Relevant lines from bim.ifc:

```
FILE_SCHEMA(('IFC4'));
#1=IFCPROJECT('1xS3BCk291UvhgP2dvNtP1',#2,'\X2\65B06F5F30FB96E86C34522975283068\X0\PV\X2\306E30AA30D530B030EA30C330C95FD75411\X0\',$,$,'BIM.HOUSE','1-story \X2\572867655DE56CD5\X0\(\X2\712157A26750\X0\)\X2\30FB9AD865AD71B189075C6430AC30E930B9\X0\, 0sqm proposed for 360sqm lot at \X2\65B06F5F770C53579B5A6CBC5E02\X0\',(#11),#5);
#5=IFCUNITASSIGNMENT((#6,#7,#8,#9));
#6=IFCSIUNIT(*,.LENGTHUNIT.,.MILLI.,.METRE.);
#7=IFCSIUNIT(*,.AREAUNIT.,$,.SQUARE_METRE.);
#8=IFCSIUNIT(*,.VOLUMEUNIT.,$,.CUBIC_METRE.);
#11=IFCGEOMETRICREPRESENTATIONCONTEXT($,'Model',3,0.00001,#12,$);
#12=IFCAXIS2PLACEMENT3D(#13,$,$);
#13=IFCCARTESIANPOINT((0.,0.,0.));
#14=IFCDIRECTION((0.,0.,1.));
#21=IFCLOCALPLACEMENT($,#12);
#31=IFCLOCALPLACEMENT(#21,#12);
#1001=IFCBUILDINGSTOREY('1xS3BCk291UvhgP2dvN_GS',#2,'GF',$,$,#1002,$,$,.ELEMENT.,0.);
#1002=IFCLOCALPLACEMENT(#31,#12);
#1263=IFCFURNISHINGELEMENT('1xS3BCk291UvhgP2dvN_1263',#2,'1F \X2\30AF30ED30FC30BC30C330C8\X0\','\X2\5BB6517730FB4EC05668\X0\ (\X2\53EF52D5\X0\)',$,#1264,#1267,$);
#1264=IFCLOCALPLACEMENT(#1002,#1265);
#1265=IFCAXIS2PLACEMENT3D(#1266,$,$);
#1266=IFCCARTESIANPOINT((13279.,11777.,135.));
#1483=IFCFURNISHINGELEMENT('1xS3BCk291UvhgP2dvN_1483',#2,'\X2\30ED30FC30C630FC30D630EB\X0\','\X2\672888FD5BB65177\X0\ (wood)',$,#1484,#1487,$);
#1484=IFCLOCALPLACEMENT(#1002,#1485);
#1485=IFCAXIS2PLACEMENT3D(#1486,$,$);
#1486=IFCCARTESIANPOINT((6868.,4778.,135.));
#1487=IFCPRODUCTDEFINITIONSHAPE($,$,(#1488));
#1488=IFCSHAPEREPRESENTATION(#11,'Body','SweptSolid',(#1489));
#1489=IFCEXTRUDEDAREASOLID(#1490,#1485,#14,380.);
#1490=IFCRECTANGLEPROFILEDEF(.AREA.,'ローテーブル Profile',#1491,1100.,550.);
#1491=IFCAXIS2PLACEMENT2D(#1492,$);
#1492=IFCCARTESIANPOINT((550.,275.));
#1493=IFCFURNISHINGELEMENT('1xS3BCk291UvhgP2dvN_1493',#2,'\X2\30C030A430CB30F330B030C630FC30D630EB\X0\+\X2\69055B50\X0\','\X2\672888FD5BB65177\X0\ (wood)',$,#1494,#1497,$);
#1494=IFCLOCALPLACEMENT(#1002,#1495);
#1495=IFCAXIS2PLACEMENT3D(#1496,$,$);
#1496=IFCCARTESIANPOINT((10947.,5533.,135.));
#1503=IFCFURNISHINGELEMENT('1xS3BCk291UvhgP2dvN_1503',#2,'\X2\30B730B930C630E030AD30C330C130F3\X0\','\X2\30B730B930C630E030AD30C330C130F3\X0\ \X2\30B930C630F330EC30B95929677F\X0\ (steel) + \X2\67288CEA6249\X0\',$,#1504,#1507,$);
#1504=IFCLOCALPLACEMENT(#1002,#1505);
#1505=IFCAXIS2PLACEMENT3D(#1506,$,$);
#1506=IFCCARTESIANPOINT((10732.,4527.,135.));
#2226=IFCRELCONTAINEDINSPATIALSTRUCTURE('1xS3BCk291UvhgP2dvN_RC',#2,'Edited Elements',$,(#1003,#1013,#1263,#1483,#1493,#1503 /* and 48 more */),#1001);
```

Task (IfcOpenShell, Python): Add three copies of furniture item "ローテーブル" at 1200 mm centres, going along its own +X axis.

```python
import ifcopenshell
import ifcopenshell.api.geometry
import ifcopenshell.api.root
import ifcopenshell.util.element
import ifcopenshell.util.placement
import ifcopenshell.util.unit

model = ifcopenshell.open("bim.ifc")
unit_scale = ifcopenshell.util.unit.calculate_unit_scale(model)


def reuse_history(source, copy):
    """copy_class also copies each property set's owner history, people and application; keep the originals."""
    for rel in copy.IsDefinedBy:
        if rel.is_a("IfcRelDefinesByProperties") and (history := rel.RelatingPropertyDefinition.OwnerHistory):
            rel.RelatingPropertyDefinition.OwnerHistory = source.OwnerHistory
            ifcopenshell.util.element.remove_deep2(model, history)


source = model.by_guid("1xS3BCk291UvhgP2dvN_1483")
base = ifcopenshell.util.placement.get_local_placement(source.ObjectPlacement)
step = base[:3, 0] * 1.2 / unit_scale

for i in range(1, 4):
    copy = ifcopenshell.api.root.copy_class(model, product=source)
    copy.Representation = ifcopenshell.util.element.copy_deep(
        model, source.Representation, exclude=["IfcGeometricRepresentationContext", "IfcRepresentationMap"]
    )
    reuse_history(source, copy)
    matrix = base.copy()
    matrix[:3, 3] += i * step
    print("added at", matrix[:3, 3].round(3) + 0.0)
    ifcopenshell.api.geometry.edit_object_placement(model, product=copy, matrix=matrix, is_si=False)

model.write("bim_v2.ifc")
```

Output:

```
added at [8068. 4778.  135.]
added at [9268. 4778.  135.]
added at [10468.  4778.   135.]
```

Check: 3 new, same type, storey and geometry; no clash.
